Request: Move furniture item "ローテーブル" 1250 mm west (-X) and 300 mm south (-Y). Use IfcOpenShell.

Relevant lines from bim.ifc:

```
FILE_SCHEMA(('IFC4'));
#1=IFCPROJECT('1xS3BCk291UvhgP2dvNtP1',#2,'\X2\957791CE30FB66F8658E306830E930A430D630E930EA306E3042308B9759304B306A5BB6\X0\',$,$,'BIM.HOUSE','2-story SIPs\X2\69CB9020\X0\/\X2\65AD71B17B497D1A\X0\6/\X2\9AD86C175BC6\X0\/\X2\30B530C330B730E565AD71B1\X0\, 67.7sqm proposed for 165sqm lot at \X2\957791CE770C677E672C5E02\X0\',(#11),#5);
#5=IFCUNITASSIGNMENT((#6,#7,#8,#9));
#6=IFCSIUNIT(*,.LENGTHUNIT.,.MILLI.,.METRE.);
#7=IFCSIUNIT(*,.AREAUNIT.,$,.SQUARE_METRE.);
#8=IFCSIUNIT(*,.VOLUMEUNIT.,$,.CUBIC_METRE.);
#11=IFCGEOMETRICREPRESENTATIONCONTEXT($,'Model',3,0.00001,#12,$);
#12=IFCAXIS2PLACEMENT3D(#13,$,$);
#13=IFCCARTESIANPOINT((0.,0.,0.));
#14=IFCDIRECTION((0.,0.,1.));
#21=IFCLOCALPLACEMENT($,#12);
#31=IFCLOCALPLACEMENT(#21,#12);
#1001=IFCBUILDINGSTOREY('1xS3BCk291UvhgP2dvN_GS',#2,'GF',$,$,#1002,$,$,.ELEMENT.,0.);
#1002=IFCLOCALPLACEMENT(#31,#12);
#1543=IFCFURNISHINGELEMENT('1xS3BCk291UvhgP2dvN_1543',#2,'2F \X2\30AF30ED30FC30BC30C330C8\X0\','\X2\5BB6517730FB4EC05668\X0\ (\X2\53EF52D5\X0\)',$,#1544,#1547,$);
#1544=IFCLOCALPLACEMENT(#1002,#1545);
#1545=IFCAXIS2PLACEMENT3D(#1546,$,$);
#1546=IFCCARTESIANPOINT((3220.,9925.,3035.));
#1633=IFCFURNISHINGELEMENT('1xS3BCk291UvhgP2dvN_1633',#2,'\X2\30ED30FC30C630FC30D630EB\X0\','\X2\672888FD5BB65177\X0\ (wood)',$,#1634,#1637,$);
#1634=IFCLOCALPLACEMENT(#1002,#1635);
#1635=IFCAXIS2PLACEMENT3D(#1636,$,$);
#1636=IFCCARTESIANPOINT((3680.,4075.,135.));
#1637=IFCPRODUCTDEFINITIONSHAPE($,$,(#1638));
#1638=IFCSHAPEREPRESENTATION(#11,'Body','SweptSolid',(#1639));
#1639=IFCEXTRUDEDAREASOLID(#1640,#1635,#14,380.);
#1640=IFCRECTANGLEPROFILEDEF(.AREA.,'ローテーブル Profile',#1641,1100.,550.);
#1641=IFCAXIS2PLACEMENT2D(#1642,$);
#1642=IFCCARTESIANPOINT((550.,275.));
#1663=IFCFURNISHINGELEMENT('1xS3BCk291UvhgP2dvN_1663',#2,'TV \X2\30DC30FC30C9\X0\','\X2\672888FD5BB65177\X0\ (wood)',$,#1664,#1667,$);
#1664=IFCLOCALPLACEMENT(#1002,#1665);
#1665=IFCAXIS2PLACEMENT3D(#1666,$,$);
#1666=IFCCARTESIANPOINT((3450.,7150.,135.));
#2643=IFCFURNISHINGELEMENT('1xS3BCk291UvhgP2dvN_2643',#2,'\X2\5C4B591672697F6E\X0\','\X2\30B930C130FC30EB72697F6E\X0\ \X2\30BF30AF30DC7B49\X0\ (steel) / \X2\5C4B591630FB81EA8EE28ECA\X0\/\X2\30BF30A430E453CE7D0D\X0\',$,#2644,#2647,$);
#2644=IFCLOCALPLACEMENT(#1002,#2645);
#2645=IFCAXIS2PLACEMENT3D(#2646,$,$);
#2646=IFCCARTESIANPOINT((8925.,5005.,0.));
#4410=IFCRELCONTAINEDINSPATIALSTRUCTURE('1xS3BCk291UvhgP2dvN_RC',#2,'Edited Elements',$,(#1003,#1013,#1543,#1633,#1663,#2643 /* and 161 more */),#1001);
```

```python
import ifcopenshell
import ifcopenshell.api.geometry
import ifcopenshell.util.placement
import ifcopenshell.util.unit

model = ifcopenshell.open("bim.ifc")
unit_scale = ifcopenshell.util.unit.calculate_unit_scale(model)

item = model.by_id(1633)
matrix = ifcopenshell.util.placement.get_local_placement(item.ObjectPlacement)
matrix[0, 3] -= 1.25 / unit_scale
matrix[1, 3] -= 0.3 / unit_scale
ifcopenshell.api.geometry.edit_object_placement(model, product=item, matrix=matrix, is_si=False)

print(ifcopenshell.util.placement.get_local_placement(item.ObjectPlacement).round(3) + 0.0)

model.write("bim_updated.ifc")
```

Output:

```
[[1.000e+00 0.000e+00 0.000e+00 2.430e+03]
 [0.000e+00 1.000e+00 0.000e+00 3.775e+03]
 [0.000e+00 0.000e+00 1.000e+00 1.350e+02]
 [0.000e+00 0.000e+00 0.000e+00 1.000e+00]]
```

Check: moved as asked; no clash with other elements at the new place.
